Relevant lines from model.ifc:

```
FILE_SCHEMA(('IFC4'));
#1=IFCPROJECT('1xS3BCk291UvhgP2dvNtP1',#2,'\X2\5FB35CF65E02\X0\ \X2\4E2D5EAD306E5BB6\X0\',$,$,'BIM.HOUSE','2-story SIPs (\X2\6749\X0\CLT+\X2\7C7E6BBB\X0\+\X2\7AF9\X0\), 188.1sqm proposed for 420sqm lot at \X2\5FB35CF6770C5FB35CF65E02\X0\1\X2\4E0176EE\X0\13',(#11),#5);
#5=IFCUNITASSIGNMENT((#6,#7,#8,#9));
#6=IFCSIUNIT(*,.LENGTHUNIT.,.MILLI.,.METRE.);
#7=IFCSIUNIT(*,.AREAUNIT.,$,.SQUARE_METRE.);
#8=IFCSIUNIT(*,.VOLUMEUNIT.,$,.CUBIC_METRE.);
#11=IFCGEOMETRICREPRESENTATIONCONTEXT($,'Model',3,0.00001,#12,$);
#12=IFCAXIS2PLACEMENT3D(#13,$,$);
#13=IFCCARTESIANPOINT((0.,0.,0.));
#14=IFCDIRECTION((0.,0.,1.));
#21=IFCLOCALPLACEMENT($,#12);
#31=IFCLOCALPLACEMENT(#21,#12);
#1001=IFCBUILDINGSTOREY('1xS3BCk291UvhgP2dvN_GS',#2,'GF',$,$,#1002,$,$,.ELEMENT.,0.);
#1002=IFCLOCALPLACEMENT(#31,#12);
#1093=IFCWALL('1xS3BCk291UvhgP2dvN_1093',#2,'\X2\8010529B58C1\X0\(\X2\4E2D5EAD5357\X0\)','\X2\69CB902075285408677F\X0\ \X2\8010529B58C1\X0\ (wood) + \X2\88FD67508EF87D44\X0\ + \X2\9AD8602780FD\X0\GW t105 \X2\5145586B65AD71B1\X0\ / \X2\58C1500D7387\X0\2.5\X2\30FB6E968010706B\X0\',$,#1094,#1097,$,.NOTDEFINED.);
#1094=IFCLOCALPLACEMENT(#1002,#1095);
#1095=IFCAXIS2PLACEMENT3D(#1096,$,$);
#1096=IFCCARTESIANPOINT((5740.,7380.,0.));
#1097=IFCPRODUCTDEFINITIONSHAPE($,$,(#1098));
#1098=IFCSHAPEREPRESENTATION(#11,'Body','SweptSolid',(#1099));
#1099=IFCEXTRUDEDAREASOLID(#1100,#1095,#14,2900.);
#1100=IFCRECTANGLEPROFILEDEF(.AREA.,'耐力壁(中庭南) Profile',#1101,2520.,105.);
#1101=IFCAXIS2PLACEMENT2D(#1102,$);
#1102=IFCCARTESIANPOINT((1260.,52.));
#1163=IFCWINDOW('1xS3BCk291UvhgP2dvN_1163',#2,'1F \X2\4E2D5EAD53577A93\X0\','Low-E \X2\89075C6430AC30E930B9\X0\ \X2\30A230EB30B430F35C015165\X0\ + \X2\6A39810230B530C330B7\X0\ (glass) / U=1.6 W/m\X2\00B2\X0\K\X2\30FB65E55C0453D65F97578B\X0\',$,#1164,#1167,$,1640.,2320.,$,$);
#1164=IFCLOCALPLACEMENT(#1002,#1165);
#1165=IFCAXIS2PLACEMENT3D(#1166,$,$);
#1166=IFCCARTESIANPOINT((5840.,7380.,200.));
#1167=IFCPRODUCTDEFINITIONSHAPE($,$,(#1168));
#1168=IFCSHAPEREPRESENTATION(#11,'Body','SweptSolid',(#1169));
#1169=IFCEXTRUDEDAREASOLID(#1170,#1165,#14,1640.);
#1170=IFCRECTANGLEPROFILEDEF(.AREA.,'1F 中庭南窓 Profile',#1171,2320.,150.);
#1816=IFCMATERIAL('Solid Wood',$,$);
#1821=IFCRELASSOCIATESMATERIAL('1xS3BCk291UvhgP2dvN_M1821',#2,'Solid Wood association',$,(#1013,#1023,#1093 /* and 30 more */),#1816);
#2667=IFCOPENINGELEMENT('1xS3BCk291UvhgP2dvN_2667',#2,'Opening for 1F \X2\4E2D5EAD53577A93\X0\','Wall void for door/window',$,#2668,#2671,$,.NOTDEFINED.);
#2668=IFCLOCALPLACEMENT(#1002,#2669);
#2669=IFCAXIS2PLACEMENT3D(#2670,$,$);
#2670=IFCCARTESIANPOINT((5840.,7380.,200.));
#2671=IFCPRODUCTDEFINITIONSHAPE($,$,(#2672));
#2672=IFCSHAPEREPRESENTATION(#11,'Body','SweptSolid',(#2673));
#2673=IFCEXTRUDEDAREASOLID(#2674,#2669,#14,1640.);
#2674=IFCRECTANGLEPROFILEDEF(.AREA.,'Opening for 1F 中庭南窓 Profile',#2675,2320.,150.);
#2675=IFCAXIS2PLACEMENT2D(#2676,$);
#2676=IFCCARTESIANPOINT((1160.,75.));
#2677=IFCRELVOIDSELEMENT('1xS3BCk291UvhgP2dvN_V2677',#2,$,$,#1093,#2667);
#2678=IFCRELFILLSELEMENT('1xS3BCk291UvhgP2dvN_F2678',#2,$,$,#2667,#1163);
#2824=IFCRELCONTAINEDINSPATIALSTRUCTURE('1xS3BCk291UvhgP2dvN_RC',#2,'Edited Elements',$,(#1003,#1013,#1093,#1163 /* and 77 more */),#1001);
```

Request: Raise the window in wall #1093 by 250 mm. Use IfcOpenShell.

```python
import numpy as np
import ifcopenshell
import ifcopenshell.api.geometry
import ifcopenshell.util.placement
import ifcopenshell.util.unit

model = ifcopenshell.open("model.ifc")
unit_scale = ifcopenshell.util.unit.calculate_unit_scale(model)

window = model.by_guid("1xS3BCk291UvhgP2dvN_1163")
opening = window.FillsVoids[0].RelatingOpeningElement
dz = 0.25 / unit_scale

shift = np.array([0.0, 0.0, dz])
# The window is not placed relative to its opening, so move both.
for product in (opening, window):
    matrix = ifcopenshell.util.placement.get_local_placement(product.ObjectPlacement)
    matrix[:3, 3] += shift
    ifcopenshell.api.geometry.edit_object_placement(model, product=product, matrix=matrix, is_si=False)

print(f"moved by {dz * unit_scale:+.3f} m")

model.write("model_rev.ifc")
```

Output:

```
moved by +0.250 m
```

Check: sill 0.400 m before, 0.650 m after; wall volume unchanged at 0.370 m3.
